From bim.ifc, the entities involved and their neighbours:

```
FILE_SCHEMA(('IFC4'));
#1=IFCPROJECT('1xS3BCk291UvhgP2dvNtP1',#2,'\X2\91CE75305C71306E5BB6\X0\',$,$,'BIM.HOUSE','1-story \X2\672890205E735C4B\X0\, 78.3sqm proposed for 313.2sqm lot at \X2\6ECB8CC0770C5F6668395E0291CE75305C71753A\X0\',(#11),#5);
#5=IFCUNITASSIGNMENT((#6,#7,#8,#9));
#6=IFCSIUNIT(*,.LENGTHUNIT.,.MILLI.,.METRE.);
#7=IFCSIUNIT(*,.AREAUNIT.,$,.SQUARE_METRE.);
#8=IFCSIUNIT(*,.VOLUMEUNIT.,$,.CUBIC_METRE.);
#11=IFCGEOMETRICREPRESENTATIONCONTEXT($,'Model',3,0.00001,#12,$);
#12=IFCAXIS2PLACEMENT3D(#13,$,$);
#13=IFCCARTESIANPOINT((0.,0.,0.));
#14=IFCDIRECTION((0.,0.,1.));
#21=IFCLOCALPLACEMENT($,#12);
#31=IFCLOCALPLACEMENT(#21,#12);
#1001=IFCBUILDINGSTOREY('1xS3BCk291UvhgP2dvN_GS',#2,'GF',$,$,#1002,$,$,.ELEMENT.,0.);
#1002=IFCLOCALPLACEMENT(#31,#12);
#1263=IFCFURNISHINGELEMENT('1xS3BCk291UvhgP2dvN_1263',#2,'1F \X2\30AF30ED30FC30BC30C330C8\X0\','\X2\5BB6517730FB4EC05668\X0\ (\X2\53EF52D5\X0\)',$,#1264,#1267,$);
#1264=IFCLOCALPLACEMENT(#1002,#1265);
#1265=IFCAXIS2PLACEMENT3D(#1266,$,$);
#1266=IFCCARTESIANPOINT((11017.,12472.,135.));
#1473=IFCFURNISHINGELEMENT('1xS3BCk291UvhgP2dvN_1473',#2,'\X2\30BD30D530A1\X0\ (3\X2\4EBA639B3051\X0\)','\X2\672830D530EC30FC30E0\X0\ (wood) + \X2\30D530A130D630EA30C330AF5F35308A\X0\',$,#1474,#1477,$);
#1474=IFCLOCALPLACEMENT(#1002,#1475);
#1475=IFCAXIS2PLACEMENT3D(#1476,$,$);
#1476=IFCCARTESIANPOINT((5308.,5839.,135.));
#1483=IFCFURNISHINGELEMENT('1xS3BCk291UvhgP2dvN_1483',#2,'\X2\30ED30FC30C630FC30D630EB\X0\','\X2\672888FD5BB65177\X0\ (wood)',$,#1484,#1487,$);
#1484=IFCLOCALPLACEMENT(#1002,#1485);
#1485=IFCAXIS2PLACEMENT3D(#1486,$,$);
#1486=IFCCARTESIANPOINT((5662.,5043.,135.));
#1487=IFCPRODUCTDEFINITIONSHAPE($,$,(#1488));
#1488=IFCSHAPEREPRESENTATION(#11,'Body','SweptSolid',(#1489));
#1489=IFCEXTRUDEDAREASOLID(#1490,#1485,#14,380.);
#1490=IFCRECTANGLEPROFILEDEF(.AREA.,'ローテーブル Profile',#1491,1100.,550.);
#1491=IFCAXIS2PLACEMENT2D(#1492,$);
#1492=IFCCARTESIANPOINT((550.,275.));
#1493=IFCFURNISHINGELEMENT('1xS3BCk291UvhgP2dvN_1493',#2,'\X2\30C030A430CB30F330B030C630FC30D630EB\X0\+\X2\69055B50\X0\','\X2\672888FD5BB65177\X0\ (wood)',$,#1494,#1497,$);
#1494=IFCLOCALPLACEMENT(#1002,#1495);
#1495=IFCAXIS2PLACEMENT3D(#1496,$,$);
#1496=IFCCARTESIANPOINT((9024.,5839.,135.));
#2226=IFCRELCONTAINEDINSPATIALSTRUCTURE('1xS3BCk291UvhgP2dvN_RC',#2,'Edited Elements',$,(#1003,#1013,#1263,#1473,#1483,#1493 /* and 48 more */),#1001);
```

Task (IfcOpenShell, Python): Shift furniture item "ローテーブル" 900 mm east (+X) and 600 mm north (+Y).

```python
import ifcopenshell
import ifcopenshell.api.geometry
import ifcopenshell.util.placement

model = ifcopenshell.open("bim.ifc")

item = model.by_guid("1xS3BCk291UvhgP2dvN_1483")
matrix = ifcopenshell.util.placement.get_local_placement(item.ObjectPlacement)
matrix[0, 3] += 900.0
matrix[1, 3] += 600.0
ifcopenshell.api.geometry.edit_object_placement(model, product=item, matrix=matrix, is_si=False)

print(ifcopenshell.util.placement.get_local_placement(item.ObjectPlacement).round(3) + 0.0)

model.write("bim_edited.ifc")
```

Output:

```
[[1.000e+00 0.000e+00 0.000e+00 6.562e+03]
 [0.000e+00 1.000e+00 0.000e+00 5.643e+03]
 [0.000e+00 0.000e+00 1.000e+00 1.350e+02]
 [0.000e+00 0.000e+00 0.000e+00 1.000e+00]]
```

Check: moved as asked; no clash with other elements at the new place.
